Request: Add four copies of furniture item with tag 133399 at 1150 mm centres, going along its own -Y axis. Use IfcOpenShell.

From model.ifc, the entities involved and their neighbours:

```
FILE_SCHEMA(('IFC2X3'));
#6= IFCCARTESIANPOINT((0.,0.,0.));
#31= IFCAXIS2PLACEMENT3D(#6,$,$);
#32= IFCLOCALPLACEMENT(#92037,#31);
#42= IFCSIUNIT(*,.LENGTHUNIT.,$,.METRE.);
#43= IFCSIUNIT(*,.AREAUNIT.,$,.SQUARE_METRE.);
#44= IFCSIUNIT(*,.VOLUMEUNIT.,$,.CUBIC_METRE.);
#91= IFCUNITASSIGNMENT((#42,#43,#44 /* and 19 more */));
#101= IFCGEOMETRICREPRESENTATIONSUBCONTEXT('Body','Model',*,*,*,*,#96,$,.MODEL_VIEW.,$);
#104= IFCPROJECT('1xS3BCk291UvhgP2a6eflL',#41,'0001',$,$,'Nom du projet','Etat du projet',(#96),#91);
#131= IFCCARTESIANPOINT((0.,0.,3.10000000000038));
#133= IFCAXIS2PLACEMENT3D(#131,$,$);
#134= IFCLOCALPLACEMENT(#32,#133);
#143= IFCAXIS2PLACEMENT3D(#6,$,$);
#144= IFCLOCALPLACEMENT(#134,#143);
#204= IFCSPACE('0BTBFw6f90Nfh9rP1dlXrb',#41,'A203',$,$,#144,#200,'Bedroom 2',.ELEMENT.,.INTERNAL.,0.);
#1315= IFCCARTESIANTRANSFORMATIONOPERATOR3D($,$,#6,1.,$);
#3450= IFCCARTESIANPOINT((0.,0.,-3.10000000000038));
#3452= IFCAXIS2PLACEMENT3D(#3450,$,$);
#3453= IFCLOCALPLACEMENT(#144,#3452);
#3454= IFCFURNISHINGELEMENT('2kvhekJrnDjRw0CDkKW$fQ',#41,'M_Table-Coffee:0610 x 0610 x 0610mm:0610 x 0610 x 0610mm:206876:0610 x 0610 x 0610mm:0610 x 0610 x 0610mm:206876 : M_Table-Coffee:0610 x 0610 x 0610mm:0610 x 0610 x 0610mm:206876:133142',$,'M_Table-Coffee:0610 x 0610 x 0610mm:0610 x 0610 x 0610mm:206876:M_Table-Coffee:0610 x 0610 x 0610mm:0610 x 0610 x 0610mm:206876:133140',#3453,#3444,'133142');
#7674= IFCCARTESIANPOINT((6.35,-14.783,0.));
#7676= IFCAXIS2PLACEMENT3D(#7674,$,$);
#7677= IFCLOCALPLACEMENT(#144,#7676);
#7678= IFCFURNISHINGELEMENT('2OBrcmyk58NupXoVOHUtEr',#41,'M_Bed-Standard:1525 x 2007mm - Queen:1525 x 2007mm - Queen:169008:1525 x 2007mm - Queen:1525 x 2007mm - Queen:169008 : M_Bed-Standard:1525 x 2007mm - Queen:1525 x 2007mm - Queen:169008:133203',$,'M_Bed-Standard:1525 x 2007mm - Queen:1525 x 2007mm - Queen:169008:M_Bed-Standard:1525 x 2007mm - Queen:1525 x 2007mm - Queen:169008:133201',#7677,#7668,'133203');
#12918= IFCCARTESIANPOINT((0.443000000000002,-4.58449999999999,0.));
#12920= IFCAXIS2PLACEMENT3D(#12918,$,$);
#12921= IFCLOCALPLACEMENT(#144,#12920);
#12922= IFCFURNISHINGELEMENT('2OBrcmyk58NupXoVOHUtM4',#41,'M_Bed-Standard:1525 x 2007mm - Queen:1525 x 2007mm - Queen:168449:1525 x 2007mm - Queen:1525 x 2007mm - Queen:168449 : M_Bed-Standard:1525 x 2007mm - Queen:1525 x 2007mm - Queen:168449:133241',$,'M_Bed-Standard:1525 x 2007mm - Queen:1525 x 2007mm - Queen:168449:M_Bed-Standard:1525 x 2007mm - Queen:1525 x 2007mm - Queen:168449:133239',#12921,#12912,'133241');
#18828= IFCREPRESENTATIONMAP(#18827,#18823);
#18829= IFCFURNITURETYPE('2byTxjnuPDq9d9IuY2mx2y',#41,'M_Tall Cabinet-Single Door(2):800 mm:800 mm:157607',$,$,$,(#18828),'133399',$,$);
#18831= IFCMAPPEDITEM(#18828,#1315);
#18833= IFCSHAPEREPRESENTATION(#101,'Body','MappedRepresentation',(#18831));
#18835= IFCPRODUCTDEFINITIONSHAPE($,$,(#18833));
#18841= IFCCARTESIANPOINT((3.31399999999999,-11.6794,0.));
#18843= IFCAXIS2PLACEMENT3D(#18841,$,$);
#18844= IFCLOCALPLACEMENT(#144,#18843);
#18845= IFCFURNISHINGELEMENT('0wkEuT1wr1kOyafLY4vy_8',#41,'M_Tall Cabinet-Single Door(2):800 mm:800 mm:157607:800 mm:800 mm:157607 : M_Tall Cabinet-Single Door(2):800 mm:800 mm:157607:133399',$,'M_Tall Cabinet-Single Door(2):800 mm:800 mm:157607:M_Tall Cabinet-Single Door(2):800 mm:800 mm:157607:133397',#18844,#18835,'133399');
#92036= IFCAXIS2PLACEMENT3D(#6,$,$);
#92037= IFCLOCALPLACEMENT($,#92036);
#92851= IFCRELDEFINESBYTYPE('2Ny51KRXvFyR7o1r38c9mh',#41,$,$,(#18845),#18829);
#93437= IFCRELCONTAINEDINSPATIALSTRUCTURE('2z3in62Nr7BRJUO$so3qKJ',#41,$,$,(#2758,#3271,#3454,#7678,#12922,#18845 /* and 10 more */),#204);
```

```python
import ifcopenshell
import ifcopenshell.api.geometry
import ifcopenshell.api.root
import ifcopenshell.util.element
import ifcopenshell.util.placement
import ifcopenshell.util.unit

model = ifcopenshell.open("model.ifc")
unit_scale = ifcopenshell.util.unit.calculate_unit_scale(model)

source = model.by_id(18845)
base = ifcopenshell.util.placement.get_local_placement(source.ObjectPlacement)
step = -base[:3, 1] * 1.15 / unit_scale

for i in range(1, 5):
    copy = ifcopenshell.api.root.copy_class(model, product=source)
    copy.Representation = ifcopenshell.util.element.copy_deep(
        model, source.Representation, exclude=["IfcGeometricRepresentationContext", "IfcRepresentationMap"]
    )
    copy.Name = "M_Tall Cabinet-Single Door(2):800 mm:800 mm:157607:800 mm:800 mm:157607 : M_Tall Cabinet-Single Door(2):800 mm:800 mm"
    copy.Tag = None
    matrix = base.copy()
    matrix[:3, 3] += i * step
    print("added at", matrix[:3, 3].round(3) + 0.0)
    ifcopenshell.api.geometry.edit_object_placement(model, product=copy, matrix=matrix, is_si=False)

model.write("model_edited.ifc")
```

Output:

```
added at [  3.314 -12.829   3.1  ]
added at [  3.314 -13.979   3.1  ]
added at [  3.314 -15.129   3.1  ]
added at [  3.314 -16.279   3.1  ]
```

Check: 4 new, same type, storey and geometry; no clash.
